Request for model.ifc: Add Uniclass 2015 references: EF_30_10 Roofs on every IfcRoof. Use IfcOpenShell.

First a look at what the model holds.

```python
import ifcopenshell

model = ifcopenshell.open("model.ifc")
print(model.schema)
print("classifications:", [c.Name for c in model.by_type("IfcClassification")])
for ifc_class in ("IfcDoor", "IfcRoof", "IfcStair", "IfcWall", "IfcWindow"):
    print(ifc_class, len(model.by_type(ifc_class)))
```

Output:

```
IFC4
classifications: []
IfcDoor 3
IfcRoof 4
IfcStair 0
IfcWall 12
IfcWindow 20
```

```python
import ifcopenshell
import ifcopenshell.api.classification

model = ifcopenshell.open("model.ifc")

system = ifcopenshell.api.classification.add_classification(model, classification="Uniclass 2015")

codes = {
    "IfcRoof": ("EF_30_10", "Roofs"),
}
for ifc_class, (code, name) in codes.items():
    products = model.by_type(ifc_class)
    ifcopenshell.api.classification.add_reference(
        model, products=products, classification=system, identification=code, name=name
    )
    print(code, len(products))

model.write("model_rev.ifc")
```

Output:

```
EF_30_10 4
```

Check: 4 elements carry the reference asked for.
